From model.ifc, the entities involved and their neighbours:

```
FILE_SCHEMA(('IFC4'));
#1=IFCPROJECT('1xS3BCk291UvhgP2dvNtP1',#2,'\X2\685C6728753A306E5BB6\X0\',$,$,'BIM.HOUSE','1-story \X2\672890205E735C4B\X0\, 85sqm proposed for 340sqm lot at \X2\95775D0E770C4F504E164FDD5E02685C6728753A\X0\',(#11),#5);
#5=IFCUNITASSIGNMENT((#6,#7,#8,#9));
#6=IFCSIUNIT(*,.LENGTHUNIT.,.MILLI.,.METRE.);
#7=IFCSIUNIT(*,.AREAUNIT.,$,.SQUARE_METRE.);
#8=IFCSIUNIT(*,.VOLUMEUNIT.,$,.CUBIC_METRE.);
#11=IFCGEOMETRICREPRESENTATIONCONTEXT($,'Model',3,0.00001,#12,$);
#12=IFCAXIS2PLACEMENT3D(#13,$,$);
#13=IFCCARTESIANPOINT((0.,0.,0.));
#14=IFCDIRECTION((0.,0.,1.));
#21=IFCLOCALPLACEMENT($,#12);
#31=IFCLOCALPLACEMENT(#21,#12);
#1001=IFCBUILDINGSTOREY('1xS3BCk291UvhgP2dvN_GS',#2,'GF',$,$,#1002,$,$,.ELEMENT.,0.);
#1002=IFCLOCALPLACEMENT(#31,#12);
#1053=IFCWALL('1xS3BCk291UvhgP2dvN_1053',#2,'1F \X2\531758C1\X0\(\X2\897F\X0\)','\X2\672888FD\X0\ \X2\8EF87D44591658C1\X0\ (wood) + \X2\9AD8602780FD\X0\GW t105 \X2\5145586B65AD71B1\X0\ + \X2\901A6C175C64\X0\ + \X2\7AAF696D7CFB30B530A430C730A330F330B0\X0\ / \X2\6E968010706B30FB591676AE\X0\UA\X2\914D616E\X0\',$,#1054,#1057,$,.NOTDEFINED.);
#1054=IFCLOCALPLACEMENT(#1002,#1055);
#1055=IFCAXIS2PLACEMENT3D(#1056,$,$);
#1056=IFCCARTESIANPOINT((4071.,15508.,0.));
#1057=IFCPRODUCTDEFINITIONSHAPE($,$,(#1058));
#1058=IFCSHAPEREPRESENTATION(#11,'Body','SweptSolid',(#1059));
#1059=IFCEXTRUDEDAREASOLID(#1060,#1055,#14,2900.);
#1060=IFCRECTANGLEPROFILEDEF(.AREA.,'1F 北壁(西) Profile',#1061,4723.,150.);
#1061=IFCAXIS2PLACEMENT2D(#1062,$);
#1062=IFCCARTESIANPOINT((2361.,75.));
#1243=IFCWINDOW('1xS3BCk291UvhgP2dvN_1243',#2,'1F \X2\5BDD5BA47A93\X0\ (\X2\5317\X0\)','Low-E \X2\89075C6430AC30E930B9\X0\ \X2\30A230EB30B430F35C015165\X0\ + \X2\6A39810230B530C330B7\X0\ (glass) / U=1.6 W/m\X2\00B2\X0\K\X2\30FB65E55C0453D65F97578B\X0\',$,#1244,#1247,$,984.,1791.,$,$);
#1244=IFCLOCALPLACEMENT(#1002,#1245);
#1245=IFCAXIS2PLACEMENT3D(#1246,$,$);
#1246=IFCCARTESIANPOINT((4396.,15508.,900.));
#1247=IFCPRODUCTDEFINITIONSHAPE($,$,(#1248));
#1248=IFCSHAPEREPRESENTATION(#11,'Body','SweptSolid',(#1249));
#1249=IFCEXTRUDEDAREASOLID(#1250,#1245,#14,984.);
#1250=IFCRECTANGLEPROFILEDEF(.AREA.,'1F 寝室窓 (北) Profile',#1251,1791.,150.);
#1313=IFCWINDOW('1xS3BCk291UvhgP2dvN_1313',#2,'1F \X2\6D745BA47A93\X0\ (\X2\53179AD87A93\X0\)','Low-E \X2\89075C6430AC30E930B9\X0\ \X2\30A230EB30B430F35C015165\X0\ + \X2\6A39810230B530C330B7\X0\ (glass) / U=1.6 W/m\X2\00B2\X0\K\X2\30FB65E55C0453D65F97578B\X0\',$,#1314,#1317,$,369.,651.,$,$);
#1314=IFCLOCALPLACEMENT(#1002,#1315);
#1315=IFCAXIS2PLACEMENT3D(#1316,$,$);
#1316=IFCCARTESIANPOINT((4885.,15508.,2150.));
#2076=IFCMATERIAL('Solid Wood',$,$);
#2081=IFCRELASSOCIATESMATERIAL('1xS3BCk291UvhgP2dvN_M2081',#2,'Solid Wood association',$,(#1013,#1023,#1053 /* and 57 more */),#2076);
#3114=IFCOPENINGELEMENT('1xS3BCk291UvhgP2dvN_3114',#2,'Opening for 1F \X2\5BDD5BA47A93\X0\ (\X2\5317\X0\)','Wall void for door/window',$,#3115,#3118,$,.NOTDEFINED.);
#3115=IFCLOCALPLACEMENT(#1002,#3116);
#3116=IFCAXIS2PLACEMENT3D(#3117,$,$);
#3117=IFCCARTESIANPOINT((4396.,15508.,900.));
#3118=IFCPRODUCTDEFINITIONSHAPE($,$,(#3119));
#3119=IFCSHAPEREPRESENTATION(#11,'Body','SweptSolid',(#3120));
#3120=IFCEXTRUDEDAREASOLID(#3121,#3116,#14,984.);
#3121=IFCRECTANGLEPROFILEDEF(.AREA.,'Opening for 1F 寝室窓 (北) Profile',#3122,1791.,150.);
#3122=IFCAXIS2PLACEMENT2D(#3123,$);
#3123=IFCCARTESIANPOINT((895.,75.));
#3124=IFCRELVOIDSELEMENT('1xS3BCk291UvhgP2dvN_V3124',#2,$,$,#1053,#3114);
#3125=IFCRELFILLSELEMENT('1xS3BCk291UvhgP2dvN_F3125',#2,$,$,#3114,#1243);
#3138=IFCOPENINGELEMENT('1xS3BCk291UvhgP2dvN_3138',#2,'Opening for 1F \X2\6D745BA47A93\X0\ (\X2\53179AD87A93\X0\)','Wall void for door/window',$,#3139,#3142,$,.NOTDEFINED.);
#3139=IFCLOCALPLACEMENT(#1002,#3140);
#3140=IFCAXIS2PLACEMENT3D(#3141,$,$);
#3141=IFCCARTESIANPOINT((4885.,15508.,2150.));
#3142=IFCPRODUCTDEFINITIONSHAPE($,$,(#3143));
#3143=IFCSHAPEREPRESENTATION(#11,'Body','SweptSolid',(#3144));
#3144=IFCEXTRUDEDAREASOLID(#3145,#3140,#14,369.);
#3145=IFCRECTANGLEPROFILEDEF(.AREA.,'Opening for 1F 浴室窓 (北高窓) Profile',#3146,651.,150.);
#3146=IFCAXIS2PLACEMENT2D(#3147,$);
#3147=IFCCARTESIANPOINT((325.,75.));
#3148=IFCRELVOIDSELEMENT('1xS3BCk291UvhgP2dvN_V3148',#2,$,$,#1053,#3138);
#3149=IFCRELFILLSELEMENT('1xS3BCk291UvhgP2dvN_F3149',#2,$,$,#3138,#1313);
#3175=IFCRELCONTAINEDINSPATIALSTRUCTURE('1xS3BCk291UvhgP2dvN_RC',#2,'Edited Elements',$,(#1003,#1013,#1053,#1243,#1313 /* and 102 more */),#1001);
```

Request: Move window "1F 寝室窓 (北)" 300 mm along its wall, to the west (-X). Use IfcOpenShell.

```python
import ifcopenshell
import ifcopenshell.api.geometry
import ifcopenshell.util.placement
import ifcopenshell.util.unit

model = ifcopenshell.open("model.ifc")
unit_scale = ifcopenshell.util.unit.calculate_unit_scale(model)

window = model.by_guid("1xS3BCk291UvhgP2dvN_1243")
opening = window.FillsVoids[0].RelatingOpeningElement
wall = opening.VoidsElements[0].RelatingBuildingElement

wall_matrix = ifcopenshell.util.placement.get_local_placement(wall.ObjectPlacement)
shift = wall_matrix[:3, 0] * -0.3 / unit_scale
before = ifcopenshell.util.placement.get_local_placement(window.ObjectPlacement)[:3, 3].copy()

# The window is not placed relative to its opening, so move both.
for product in (opening, window):
    matrix = ifcopenshell.util.placement.get_local_placement(product.ObjectPlacement)
    matrix[:3, 3] += shift
    ifcopenshell.api.geometry.edit_object_placement(model, product=product, matrix=matrix, is_si=False)

after = ifcopenshell.util.placement.get_local_placement(window.ObjectPlacement)[:3, 3]
print("window moved by", (after - before).round(3) + 0.0)

model.write("model-out.ifc")
```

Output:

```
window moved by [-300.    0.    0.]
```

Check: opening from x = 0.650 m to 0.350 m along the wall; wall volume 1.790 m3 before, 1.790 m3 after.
